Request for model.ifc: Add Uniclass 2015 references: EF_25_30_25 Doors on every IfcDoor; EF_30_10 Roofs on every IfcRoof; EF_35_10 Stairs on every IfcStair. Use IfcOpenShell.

First a look at what the model holds.

```python
import ifcopenshell

model = ifcopenshell.open("model.ifc")
print(model.schema)
print("classifications:", [c.Name for c in model.by_type("IfcClassification")])
for ifc_class in ("IfcDoor", "IfcRoof", "IfcStair", "IfcWall", "IfcWindow"):
    print(ifc_class, len(model.by_type(ifc_class)))
```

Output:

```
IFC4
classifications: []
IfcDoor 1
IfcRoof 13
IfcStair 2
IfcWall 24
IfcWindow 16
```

```python
import ifcopenshell
import ifcopenshell.api.classification

model = ifcopenshell.open("model.ifc")

system = ifcopenshell.api.classification.add_classification(model, classification="Uniclass 2015")

codes = {
    "IfcDoor": ("EF_25_30_25", "Doors"),
    "IfcRoof": ("EF_30_10", "Roofs"),
    "IfcStair": ("EF_35_10", "Stairs"),
}
for ifc_class, (code, name) in codes.items():
    products = model.by_type(ifc_class)
    ifcopenshell.api.classification.add_reference(
        model, products=products, classification=system, identification=code, name=name
    )
    print(code, len(products))

model.write("model_rev.ifc")
```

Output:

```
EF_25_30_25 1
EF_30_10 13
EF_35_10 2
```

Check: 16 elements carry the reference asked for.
